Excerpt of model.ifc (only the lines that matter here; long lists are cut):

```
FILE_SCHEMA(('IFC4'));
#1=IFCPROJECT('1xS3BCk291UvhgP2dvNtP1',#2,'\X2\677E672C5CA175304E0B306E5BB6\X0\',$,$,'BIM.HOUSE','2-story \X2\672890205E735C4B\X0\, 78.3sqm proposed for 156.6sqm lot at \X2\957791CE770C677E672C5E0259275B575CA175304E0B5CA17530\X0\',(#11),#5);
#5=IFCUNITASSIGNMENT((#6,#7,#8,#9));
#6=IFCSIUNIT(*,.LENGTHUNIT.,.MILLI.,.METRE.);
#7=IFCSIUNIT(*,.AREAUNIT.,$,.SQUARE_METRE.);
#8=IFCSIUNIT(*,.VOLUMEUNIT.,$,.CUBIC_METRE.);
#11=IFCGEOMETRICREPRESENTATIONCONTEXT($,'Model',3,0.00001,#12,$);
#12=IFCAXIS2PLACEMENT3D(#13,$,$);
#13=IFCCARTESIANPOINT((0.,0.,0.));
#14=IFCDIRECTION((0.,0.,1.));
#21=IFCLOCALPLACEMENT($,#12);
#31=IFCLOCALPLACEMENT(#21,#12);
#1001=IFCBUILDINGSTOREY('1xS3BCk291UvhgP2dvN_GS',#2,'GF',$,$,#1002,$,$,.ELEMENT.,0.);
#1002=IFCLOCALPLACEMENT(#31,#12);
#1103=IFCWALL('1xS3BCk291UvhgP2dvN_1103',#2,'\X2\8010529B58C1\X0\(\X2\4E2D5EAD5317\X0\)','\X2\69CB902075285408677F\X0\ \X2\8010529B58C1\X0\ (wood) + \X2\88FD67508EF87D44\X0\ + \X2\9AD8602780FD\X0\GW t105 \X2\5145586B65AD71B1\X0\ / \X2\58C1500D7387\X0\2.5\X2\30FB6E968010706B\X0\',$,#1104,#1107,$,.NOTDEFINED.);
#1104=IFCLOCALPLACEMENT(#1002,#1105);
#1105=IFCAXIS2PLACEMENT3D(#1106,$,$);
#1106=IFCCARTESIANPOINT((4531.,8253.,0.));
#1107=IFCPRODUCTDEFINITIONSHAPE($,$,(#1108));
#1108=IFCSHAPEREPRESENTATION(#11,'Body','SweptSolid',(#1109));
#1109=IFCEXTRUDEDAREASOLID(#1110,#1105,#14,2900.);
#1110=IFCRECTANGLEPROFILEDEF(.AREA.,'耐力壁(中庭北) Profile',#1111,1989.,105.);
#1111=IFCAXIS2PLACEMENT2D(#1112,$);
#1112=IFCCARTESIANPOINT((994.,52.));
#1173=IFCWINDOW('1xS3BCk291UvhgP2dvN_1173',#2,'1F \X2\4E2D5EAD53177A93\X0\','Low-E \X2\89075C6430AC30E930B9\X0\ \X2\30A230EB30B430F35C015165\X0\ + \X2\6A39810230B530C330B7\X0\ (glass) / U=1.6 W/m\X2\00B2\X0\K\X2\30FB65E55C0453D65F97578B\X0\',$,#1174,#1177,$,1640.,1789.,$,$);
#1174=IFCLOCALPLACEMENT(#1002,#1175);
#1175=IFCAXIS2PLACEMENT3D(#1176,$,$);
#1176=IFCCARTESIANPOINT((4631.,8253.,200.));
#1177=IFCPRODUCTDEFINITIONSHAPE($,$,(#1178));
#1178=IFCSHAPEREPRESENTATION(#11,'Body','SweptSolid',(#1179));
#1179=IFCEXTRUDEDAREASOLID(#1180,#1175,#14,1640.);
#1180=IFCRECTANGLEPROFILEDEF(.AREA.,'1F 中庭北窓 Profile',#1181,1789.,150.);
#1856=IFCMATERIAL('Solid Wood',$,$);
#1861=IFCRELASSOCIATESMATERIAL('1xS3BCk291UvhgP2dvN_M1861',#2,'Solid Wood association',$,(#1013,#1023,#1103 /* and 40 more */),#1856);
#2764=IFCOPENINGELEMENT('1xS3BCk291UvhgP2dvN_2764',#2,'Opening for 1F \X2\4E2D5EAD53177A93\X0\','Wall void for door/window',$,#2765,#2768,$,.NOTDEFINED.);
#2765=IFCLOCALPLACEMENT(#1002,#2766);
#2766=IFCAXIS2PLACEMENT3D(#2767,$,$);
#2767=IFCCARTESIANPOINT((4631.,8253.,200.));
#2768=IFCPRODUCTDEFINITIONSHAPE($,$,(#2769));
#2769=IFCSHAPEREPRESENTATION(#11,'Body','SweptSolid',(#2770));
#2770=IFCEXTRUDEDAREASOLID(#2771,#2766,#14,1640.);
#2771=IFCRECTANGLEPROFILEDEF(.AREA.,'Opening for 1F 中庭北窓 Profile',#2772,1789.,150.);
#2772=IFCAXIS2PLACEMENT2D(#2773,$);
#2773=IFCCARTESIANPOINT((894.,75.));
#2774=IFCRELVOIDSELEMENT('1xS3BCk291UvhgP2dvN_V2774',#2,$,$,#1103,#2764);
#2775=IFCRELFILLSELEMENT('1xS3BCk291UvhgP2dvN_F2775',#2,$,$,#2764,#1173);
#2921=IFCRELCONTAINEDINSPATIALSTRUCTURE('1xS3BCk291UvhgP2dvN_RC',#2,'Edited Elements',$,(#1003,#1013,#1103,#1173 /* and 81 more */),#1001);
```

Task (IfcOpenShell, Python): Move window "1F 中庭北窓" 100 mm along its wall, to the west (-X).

```python
import ifcopenshell
import ifcopenshell.api.geometry
import ifcopenshell.util.placement
import ifcopenshell.util.unit

model = ifcopenshell.open("model.ifc")
unit_scale = ifcopenshell.util.unit.calculate_unit_scale(model)

window = model.by_guid("1xS3BCk291UvhgP2dvN_1173")
opening = window.FillsVoids[0].RelatingOpeningElement
wall = opening.VoidsElements[0].RelatingBuildingElement

wall_matrix = ifcopenshell.util.placement.get_local_placement(wall.ObjectPlacement)
shift = wall_matrix[:3, 0] * -0.1 / unit_scale
before = ifcopenshell.util.placement.get_local_placement(window.ObjectPlacement)[:3, 3].copy()

# The window is not placed relative to its opening, so move both.
for product in (opening, window):
    matrix = ifcopenshell.util.placement.get_local_placement(product.ObjectPlacement)
    matrix[:3, 3] += shift
    ifcopenshell.api.geometry.edit_object_placement(model, product=product, matrix=matrix, is_si=False)

after = ifcopenshell.util.placement.get_local_placement(window.ObjectPlacement)[:3, 3]
print("window moved by", (after - before).round(3) + 0.0)

model.write("model_updated.ifc")
```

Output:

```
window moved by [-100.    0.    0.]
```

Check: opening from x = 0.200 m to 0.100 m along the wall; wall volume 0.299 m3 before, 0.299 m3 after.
